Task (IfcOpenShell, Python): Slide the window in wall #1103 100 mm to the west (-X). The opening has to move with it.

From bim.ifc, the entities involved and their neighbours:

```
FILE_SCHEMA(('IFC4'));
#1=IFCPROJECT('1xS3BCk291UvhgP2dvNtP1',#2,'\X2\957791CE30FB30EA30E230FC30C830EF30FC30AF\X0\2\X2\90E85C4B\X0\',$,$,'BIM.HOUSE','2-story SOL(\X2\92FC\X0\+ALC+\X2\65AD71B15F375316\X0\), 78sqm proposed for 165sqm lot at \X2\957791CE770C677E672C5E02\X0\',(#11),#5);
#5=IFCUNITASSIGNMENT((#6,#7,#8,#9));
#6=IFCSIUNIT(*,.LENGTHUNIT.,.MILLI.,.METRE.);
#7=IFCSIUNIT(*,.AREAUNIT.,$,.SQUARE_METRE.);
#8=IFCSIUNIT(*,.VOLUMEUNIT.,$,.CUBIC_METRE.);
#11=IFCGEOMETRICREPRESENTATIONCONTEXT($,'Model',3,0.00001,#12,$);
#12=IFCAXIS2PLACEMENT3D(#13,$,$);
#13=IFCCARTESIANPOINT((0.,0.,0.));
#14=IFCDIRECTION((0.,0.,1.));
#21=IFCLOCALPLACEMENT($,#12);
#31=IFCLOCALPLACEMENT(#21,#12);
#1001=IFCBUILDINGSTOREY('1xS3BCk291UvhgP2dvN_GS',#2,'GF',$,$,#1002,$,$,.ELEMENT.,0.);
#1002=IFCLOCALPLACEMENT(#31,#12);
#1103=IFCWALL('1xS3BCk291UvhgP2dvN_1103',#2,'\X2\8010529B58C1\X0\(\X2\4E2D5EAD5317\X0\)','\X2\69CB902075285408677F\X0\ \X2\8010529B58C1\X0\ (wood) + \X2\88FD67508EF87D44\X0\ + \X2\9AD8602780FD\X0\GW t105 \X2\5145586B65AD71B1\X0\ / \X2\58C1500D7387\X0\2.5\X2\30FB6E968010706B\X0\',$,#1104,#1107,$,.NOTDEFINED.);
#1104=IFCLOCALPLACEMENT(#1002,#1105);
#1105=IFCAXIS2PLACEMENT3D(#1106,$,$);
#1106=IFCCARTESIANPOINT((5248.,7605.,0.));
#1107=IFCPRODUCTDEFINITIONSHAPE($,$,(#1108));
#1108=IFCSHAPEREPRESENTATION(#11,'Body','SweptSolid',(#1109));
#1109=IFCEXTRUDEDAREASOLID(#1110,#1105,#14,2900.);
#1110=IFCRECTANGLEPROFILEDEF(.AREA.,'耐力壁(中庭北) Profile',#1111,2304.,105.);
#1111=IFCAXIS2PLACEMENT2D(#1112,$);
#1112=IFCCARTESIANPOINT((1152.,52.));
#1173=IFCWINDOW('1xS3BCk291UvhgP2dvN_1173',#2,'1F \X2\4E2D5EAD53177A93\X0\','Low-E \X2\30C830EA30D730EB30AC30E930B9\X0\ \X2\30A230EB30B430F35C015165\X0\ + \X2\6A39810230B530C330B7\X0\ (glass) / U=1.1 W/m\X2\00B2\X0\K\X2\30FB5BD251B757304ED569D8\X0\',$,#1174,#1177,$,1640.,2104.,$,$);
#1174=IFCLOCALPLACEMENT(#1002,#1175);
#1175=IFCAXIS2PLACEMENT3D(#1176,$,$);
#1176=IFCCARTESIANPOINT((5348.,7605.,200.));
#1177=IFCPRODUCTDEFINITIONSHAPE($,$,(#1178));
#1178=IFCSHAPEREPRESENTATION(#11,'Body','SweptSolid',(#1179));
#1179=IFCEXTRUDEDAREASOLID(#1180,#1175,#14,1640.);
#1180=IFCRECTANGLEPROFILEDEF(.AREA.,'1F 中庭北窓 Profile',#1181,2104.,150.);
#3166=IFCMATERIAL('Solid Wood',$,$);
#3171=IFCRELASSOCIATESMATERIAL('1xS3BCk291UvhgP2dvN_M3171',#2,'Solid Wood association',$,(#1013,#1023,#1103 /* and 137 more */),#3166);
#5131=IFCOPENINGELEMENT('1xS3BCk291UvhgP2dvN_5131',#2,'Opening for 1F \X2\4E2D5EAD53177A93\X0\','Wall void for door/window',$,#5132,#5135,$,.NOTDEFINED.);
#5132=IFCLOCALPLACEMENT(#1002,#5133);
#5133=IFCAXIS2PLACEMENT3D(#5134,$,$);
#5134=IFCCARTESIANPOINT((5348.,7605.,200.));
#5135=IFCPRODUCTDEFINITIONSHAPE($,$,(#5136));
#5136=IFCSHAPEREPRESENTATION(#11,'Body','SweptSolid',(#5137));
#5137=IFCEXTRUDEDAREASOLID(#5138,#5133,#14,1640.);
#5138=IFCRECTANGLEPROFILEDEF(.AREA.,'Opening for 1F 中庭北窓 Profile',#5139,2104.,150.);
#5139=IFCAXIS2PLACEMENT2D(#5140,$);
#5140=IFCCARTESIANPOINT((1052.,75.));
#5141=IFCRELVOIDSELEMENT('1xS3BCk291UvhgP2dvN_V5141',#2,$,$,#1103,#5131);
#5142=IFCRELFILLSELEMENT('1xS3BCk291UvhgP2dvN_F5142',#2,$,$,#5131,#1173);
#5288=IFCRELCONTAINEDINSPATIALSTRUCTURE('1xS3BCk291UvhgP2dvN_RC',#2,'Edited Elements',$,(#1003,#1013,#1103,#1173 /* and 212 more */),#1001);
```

```python
import ifcopenshell
import ifcopenshell.api.geometry
import ifcopenshell.util.placement

model = ifcopenshell.open("bim.ifc")

window = model.by_id(1173)
opening = window.FillsVoids[0].RelatingOpeningElement
wall = opening.VoidsElements[0].RelatingBuildingElement

wall_matrix = ifcopenshell.util.placement.get_local_placement(wall.ObjectPlacement)
shift = wall_matrix[:3, 0] * -100.0
before = ifcopenshell.util.placement.get_local_placement(window.ObjectPlacement)[:3, 3].copy()

# The window is not placed relative to its opening, so move both.
for product in (opening, window):
    matrix = ifcopenshell.util.placement.get_local_placement(product.ObjectPlacement)
    matrix[:3, 3] += shift
    ifcopenshell.api.geometry.edit_object_placement(model, product=product, matrix=matrix, is_si=False)

after = ifcopenshell.util.placement.get_local_placement(window.ObjectPlacement)[:3, 3]
print("window moved by", (after - before).round(3) + 0.0)

model.write("bim_edited.ifc")
```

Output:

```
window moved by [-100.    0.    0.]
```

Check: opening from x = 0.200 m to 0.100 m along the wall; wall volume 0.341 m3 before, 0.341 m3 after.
